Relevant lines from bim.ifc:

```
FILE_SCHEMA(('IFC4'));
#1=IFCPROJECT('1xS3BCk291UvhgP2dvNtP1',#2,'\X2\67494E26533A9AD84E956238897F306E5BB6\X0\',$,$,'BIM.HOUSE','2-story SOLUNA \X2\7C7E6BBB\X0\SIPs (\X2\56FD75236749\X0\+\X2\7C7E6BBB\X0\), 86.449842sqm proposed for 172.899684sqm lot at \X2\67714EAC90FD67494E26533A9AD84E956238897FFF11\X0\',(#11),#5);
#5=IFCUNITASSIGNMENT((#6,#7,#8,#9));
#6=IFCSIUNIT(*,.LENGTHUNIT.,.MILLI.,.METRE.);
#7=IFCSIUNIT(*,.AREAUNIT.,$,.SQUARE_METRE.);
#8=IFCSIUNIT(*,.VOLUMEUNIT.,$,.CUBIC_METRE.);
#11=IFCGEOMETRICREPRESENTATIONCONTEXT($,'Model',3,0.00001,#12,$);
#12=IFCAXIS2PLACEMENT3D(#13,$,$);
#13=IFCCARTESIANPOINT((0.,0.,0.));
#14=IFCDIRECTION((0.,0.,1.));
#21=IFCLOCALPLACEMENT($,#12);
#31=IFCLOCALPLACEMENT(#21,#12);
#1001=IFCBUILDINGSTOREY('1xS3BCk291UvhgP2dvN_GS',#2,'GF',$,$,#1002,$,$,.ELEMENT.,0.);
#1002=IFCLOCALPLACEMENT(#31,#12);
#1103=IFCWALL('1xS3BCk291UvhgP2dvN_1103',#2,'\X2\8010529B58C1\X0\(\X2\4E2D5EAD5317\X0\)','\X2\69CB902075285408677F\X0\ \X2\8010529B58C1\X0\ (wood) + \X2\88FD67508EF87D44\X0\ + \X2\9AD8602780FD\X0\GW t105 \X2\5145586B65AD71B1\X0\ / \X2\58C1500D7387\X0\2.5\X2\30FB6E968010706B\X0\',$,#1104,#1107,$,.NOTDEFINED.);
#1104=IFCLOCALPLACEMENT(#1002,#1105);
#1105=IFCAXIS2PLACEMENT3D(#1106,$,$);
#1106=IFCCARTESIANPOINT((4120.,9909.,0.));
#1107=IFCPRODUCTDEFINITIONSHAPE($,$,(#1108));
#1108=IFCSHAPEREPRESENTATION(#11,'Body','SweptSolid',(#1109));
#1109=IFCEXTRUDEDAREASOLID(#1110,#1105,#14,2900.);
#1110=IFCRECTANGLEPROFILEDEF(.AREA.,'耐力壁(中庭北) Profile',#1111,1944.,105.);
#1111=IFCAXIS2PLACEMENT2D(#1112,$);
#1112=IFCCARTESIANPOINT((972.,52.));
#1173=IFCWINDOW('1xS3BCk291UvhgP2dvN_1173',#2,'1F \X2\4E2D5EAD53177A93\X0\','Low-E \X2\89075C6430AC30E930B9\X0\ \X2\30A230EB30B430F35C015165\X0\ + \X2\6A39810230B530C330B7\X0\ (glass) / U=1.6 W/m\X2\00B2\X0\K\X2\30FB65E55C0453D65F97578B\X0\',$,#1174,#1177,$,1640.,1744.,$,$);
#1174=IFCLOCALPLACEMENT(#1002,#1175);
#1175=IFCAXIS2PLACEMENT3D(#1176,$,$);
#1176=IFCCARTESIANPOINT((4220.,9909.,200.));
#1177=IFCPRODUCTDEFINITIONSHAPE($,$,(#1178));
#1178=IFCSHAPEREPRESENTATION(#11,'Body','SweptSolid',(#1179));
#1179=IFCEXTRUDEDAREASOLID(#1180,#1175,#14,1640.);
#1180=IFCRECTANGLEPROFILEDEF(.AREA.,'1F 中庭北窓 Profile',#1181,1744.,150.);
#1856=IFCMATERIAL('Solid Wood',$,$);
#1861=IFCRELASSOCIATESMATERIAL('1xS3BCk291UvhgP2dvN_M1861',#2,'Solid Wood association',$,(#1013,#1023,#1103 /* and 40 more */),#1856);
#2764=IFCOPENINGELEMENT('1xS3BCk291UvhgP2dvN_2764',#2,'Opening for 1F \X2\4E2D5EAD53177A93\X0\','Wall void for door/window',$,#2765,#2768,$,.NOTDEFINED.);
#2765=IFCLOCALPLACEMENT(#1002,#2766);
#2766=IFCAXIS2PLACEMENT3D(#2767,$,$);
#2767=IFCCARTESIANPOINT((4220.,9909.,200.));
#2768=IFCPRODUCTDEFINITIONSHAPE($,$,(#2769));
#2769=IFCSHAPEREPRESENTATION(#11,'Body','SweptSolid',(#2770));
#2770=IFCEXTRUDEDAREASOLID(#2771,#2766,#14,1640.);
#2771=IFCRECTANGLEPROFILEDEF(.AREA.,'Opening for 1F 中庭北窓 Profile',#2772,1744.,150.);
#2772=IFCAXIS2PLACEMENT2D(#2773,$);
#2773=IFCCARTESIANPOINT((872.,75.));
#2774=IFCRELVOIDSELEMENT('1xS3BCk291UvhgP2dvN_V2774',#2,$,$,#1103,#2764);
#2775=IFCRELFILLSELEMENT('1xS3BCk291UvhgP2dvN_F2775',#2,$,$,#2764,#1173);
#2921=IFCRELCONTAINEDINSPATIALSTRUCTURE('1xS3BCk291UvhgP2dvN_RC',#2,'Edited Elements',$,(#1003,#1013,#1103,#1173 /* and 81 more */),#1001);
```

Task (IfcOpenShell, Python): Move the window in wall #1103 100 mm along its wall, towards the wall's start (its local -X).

```python
import ifcopenshell
import ifcopenshell.api.geometry
import ifcopenshell.util.placement

model = ifcopenshell.open("bim.ifc")

window = model.by_guid("1xS3BCk291UvhgP2dvN_1173")
opening = window.FillsVoids[0].RelatingOpeningElement
wall = opening.VoidsElements[0].RelatingBuildingElement

wall_matrix = ifcopenshell.util.placement.get_local_placement(wall.ObjectPlacement)
shift = wall_matrix[:3, 0] * -100.0
before = ifcopenshell.util.placement.get_local_placement(window.ObjectPlacement)[:3, 3].copy()

# The window is not placed relative to its opening, so move both.
for product in (opening, window):
    matrix = ifcopenshell.util.placement.get_local_placement(product.ObjectPlacement)
    matrix[:3, 3] += shift
    ifcopenshell.api.geometry.edit_object_placement(model, product=product, matrix=matrix, is_si=False)

after = ifcopenshell.util.placement.get_local_placement(window.ObjectPlacement)[:3, 3]
print("window moved by", (after - before).round(3) + 0.0)

model.write("bim_updated.ifc")
```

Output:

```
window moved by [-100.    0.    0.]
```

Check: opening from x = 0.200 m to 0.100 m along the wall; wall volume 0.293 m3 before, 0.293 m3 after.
